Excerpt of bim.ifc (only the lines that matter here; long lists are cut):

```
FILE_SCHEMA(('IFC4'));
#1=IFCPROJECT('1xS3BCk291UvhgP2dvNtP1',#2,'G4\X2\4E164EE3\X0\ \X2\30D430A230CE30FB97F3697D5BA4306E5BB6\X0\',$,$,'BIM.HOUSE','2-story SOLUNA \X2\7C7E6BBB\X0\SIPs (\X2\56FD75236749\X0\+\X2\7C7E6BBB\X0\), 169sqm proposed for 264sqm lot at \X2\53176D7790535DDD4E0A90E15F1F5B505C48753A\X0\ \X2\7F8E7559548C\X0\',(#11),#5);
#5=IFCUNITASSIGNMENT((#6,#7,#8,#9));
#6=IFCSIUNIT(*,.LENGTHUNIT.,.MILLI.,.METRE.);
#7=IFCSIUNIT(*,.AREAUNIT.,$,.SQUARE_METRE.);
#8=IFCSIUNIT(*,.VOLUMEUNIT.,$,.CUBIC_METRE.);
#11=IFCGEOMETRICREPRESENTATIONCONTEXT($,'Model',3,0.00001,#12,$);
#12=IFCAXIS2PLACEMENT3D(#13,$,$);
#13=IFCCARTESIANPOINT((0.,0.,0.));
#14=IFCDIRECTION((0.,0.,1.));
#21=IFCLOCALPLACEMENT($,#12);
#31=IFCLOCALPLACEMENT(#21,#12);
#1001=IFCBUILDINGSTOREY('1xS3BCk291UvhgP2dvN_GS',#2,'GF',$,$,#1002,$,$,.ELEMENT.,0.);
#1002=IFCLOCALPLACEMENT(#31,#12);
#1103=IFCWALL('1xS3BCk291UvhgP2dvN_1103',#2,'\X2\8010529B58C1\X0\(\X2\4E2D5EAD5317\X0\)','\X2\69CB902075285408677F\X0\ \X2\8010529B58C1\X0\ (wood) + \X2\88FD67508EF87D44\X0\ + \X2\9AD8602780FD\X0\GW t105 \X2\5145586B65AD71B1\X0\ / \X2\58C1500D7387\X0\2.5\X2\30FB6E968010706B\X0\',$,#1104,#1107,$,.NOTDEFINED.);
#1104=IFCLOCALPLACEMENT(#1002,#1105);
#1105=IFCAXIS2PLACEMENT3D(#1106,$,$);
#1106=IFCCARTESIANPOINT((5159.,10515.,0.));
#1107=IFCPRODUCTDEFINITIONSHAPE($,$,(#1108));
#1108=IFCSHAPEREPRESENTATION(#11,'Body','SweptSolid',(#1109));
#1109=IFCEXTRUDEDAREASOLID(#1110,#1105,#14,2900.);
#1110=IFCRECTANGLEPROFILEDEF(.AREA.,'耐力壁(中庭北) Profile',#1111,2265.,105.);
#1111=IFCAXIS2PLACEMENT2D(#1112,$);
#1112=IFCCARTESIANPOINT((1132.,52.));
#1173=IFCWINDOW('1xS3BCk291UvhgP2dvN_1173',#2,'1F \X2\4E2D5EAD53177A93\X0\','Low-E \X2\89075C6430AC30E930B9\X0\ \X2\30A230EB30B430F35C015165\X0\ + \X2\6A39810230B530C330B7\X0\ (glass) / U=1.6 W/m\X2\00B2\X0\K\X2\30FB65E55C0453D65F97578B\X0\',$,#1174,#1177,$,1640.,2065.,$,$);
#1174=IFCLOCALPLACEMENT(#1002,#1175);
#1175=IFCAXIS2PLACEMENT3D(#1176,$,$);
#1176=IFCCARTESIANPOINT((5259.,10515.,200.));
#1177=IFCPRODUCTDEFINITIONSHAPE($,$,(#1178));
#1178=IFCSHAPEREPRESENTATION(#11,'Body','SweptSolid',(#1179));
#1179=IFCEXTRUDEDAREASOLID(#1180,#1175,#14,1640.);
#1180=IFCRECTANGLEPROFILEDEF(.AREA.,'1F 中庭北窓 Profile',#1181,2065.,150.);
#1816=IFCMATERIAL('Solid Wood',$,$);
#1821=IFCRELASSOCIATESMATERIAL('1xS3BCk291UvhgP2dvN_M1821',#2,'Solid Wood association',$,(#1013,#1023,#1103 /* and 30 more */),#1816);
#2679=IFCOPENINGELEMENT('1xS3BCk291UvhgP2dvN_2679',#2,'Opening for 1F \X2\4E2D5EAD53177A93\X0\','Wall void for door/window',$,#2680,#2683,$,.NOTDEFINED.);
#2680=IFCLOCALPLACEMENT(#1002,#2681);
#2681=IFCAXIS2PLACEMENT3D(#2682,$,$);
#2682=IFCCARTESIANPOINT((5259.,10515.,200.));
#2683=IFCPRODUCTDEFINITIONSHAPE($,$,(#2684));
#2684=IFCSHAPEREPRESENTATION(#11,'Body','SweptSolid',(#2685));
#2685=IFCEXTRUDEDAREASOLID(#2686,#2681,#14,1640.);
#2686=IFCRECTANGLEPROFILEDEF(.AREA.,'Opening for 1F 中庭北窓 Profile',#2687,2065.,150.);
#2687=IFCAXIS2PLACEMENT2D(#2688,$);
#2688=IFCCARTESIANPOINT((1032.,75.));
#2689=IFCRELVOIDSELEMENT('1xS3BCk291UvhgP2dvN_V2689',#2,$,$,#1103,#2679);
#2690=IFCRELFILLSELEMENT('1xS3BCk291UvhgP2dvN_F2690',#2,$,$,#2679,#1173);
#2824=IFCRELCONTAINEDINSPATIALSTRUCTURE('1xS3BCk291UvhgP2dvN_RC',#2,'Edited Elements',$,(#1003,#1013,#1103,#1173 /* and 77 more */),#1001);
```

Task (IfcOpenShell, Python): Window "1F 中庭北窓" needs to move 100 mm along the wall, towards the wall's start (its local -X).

```python
import ifcopenshell
import ifcopenshell.api.geometry
import ifcopenshell.util.placement

model = ifcopenshell.open("bim.ifc")

window = model.by_guid("1xS3BCk291UvhgP2dvN_1173")
opening = window.FillsVoids[0].RelatingOpeningElement
wall = opening.VoidsElements[0].RelatingBuildingElement

wall_matrix = ifcopenshell.util.placement.get_local_placement(wall.ObjectPlacement)
shift = wall_matrix[:3, 0] * -100.0
before = ifcopenshell.util.placement.get_local_placement(window.ObjectPlacement)[:3, 3].copy()

# The window is not placed relative to its opening, so move both.
for product in (opening, window):
    matrix = ifcopenshell.util.placement.get_local_placement(product.ObjectPlacement)
    matrix[:3, 3] += shift
    ifcopenshell.api.geometry.edit_object_placement(model, product=product, matrix=matrix, is_si=False)

after = ifcopenshell.util.placement.get_local_placement(window.ObjectPlacement)[:3, 3]
print("window moved by", (after - before).round(3) + 0.0)

model.write("bim-out.ifc")
```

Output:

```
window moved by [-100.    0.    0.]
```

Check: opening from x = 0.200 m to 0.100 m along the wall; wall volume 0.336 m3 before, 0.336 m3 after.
